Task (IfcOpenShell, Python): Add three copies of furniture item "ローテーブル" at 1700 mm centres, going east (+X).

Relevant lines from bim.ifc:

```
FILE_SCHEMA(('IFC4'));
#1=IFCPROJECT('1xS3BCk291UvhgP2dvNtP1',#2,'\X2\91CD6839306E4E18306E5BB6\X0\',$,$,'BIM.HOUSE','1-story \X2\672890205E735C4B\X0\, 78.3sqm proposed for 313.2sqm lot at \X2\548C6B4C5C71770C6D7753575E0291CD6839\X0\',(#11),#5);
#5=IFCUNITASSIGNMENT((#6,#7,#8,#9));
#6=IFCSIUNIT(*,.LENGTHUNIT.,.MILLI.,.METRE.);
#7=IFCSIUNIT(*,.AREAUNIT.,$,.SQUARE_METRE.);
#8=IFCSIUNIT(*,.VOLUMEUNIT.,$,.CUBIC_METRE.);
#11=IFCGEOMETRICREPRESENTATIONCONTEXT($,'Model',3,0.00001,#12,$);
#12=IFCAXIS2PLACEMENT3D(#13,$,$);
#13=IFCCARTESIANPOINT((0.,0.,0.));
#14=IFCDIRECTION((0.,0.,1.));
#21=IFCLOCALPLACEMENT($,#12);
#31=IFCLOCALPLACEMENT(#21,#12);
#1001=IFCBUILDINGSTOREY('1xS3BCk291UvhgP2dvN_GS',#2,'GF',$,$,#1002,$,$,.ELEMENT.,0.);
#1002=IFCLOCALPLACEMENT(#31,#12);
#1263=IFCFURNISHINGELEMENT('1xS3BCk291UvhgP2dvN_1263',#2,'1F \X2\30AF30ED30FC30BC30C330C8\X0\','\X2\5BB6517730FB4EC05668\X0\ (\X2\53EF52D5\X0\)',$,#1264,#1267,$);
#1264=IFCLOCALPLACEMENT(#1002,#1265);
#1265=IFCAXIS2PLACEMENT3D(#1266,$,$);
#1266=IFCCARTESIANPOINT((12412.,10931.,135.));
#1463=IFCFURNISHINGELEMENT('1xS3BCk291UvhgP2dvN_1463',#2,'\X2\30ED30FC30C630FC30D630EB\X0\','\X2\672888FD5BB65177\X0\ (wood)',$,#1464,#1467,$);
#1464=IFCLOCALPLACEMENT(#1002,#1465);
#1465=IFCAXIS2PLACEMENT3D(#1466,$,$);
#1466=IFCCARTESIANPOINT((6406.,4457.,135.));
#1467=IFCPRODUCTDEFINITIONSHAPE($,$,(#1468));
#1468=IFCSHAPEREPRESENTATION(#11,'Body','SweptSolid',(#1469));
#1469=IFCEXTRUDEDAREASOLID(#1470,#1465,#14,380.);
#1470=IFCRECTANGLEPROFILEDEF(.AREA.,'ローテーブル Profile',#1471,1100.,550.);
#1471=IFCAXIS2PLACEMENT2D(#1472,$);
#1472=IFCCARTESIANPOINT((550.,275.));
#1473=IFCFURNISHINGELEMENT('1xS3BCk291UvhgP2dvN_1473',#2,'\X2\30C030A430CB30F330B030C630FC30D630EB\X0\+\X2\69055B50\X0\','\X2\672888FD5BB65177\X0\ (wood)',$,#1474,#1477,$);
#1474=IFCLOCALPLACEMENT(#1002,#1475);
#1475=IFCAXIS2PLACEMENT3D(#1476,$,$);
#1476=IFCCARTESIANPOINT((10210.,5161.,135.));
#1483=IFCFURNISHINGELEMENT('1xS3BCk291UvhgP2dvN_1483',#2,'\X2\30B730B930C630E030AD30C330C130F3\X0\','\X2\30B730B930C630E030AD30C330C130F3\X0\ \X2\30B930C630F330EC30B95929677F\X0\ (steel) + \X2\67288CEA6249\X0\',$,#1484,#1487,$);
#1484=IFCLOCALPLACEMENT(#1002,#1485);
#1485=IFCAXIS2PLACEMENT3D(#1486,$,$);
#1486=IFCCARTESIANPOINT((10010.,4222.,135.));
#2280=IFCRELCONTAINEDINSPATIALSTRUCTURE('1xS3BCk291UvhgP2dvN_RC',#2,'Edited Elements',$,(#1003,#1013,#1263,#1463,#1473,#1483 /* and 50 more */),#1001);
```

```python
import numpy as np
import ifcopenshell
import ifcopenshell.api.geometry
import ifcopenshell.api.root
import ifcopenshell.util.element
import ifcopenshell.util.placement
import ifcopenshell.util.unit

model = ifcopenshell.open("bim.ifc")
unit_scale = ifcopenshell.util.unit.calculate_unit_scale(model)


def reuse_history(source, copy):
    """copy_class also copies each property set's owner history, people and application; keep the originals."""
    for rel in copy.IsDefinedBy:
        if rel.is_a("IfcRelDefinesByProperties") and (history := rel.RelatingPropertyDefinition.OwnerHistory):
            rel.RelatingPropertyDefinition.OwnerHistory = source.OwnerHistory
            ifcopenshell.util.element.remove_deep2(model, history)


source = model.by_id(1463)
base = ifcopenshell.util.placement.get_local_placement(source.ObjectPlacement)
step = np.array([1.0, 0.0, 0.0]) * 1.7 / unit_scale

for i in range(1, 4):
    copy = ifcopenshell.api.root.copy_class(model, product=source)
    copy.Representation = ifcopenshell.util.element.copy_deep(
        model, source.Representation, exclude=["IfcGeometricRepresentationContext", "IfcRepresentationMap"]
    )
    reuse_history(source, copy)
    matrix = base.copy()
    matrix[:3, 3] += i * step
    print("added at", matrix[:3, 3].round(3) + 0.0)
    ifcopenshell.api.geometry.edit_object_placement(model, product=copy, matrix=matrix, is_si=False)

model.write("bim_updated.ifc")
```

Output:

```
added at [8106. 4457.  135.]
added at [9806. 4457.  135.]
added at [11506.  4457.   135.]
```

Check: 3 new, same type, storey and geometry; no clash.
